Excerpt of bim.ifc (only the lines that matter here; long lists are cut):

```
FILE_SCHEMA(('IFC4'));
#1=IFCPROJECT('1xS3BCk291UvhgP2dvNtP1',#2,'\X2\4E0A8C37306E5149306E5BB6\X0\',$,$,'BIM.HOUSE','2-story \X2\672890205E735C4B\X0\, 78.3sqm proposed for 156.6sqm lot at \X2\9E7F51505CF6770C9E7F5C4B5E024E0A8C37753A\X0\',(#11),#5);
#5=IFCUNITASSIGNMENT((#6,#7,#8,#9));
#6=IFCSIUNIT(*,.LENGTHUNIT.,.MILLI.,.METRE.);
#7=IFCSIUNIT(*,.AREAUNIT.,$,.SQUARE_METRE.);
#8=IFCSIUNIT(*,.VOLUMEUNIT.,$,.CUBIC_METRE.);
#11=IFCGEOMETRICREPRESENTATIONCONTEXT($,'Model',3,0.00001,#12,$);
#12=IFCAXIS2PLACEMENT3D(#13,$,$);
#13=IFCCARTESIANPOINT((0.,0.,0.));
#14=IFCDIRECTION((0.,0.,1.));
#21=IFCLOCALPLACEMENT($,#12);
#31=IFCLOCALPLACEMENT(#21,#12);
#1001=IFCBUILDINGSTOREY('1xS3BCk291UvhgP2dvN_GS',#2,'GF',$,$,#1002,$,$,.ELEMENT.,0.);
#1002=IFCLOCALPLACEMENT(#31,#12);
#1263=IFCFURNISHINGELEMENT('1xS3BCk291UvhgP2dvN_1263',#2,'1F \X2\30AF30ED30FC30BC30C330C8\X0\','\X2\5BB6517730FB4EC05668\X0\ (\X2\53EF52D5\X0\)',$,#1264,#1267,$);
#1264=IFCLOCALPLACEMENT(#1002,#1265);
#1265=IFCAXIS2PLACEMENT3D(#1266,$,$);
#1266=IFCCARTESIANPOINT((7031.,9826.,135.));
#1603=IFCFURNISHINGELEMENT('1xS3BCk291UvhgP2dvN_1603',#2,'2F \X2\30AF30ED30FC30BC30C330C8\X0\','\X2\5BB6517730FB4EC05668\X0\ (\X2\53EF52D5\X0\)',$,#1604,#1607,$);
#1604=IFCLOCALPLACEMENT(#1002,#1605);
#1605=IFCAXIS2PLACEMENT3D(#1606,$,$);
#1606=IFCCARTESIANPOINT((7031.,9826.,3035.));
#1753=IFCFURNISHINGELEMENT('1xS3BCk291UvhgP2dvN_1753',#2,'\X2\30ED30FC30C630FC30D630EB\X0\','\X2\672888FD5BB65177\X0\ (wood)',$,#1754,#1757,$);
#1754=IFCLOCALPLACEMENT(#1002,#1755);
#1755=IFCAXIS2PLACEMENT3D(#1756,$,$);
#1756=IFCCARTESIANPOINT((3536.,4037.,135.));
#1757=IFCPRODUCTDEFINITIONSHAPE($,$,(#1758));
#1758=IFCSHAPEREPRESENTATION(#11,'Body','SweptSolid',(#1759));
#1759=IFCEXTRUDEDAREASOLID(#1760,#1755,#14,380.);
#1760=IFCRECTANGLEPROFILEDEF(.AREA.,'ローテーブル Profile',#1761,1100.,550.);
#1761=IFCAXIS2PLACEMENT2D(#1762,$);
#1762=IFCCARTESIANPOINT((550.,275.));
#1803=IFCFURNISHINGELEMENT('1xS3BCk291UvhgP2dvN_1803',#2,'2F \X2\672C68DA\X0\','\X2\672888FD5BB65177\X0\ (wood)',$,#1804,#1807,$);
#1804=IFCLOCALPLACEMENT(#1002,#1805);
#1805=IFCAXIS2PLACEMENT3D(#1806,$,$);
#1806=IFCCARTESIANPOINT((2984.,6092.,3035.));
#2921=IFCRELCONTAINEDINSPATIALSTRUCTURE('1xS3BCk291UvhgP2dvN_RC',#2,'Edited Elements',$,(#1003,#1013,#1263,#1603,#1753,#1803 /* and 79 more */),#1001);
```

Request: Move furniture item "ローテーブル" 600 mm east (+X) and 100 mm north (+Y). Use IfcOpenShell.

```python
import ifcopenshell
import ifcopenshell.api.geometry
import ifcopenshell.util.placement

model = ifcopenshell.open("bim.ifc")

item = model.by_guid("1xS3BCk291UvhgP2dvN_1753")
matrix = ifcopenshell.util.placement.get_local_placement(item.ObjectPlacement)
matrix[0, 3] += 600.0
matrix[1, 3] += 100.0
ifcopenshell.api.geometry.edit_object_placement(model, product=item, matrix=matrix, is_si=False)

print(ifcopenshell.util.placement.get_local_placement(item.ObjectPlacement).round(3) + 0.0)

model.write("bim-out.ifc")
```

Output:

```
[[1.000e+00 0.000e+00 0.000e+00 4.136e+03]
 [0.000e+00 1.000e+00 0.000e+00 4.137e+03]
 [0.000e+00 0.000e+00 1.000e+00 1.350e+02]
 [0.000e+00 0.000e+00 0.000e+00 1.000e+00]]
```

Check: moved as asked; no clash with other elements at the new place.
